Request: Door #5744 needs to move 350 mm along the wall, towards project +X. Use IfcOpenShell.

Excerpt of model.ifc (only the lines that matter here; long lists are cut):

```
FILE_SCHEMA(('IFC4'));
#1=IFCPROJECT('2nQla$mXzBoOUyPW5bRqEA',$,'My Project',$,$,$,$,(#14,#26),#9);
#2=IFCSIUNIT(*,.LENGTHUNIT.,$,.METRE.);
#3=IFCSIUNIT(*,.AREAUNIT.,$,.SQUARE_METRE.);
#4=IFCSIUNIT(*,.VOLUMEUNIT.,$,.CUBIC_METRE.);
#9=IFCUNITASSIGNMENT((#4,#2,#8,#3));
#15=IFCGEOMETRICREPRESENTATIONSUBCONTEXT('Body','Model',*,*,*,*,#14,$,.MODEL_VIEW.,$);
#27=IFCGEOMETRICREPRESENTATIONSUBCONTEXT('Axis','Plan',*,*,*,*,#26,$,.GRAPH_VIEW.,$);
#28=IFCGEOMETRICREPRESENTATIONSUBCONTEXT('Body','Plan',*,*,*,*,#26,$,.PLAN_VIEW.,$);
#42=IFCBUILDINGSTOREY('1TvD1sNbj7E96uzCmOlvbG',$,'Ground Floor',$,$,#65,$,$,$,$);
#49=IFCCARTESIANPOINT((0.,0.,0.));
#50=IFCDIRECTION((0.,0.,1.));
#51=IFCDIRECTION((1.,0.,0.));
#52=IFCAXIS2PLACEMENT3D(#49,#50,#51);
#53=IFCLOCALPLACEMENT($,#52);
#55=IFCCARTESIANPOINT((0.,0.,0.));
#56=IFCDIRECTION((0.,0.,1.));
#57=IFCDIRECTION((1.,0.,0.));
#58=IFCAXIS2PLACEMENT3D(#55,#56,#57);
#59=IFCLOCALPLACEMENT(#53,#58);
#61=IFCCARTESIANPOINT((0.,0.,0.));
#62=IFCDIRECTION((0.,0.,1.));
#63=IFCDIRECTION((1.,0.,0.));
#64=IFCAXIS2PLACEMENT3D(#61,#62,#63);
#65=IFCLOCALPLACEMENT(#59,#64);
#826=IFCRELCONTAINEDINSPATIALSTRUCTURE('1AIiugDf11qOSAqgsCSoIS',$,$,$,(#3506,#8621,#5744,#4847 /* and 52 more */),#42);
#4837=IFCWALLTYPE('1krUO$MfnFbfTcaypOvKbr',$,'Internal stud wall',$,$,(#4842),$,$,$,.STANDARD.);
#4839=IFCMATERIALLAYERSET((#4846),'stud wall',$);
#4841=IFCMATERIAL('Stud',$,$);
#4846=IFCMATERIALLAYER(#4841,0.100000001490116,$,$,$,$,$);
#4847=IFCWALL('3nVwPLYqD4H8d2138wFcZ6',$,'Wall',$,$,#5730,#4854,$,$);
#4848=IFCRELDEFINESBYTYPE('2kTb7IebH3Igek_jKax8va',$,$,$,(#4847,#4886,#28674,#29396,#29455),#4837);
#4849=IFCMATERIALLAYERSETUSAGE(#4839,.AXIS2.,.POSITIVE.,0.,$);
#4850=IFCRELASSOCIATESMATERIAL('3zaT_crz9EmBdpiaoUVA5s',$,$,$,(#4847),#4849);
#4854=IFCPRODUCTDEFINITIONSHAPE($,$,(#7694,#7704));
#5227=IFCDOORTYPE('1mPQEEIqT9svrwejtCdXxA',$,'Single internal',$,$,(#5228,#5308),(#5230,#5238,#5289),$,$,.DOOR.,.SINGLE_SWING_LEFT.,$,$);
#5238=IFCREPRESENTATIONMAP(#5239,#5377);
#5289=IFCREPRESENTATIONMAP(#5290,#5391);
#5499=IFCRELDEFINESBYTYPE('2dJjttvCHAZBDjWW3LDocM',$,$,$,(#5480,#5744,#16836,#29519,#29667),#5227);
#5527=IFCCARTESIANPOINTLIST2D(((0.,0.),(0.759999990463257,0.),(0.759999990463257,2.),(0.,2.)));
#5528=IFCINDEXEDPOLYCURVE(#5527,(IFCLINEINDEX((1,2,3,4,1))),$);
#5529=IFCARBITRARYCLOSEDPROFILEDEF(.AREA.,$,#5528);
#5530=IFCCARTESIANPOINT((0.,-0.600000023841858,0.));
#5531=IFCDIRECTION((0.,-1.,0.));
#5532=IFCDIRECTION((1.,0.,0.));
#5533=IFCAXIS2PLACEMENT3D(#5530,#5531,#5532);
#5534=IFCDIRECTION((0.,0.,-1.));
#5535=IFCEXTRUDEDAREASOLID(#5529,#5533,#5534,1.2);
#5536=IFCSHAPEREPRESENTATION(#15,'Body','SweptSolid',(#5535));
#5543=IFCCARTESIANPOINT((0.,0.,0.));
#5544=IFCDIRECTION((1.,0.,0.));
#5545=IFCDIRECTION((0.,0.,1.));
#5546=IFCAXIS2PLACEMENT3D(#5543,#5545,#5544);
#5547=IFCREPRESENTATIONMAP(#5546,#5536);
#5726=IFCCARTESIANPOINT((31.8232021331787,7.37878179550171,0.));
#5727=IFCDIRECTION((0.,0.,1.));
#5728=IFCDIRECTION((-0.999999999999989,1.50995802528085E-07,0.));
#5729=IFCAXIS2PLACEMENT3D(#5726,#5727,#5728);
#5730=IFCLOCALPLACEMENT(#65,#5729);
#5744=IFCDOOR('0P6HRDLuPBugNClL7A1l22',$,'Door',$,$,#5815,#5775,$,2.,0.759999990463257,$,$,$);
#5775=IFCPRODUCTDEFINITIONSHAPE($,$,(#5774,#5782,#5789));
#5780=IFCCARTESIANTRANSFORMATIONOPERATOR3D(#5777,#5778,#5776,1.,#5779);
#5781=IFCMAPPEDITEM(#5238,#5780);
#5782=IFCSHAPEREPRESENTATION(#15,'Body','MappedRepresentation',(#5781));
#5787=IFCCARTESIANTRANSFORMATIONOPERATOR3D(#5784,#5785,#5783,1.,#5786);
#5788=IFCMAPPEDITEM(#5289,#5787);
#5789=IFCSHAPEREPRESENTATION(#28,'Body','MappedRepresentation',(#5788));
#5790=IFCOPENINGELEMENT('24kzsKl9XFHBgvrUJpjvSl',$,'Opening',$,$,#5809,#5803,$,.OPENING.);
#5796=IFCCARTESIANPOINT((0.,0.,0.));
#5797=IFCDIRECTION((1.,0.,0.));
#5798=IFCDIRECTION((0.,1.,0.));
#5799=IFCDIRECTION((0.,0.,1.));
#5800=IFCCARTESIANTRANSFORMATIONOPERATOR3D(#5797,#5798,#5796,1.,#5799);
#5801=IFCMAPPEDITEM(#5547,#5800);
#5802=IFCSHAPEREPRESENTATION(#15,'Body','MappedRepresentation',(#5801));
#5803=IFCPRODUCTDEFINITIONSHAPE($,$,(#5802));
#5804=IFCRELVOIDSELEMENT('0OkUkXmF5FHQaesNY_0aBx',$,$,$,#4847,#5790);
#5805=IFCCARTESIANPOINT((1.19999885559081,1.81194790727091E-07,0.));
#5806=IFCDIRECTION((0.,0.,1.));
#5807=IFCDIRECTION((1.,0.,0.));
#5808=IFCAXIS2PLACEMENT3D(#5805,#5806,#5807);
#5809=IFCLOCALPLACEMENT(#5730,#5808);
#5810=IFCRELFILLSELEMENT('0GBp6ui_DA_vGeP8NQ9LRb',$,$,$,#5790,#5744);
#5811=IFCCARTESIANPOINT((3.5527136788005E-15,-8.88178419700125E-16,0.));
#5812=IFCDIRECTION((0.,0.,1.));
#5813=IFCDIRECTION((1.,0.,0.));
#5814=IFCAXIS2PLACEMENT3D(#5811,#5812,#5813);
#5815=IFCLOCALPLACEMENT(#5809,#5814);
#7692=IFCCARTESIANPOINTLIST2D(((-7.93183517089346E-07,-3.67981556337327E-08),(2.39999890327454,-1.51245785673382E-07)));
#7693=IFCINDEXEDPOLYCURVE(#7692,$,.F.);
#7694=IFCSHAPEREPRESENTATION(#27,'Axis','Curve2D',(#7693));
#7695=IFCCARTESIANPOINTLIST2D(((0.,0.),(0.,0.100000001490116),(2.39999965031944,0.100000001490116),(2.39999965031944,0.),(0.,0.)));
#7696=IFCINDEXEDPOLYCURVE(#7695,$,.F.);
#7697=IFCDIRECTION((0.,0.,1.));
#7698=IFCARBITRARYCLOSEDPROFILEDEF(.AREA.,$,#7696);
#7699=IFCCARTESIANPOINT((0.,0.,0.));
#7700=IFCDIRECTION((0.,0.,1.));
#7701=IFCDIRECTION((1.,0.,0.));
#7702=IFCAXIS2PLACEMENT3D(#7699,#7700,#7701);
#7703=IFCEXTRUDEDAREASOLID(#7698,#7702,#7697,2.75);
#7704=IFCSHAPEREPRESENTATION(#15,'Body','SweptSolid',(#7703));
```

```python
import ifcopenshell
import ifcopenshell.api.geometry
import ifcopenshell.util.placement

model = ifcopenshell.open("model.ifc")

door = model.by_guid("0P6HRDLuPBugNClL7A1l22")
opening = door.FillsVoids[0].RelatingOpeningElement
wall = opening.VoidsElements[0].RelatingBuildingElement

wall_matrix = ifcopenshell.util.placement.get_local_placement(wall.ObjectPlacement)
shift = wall_matrix[:3, 0] * -0.35
before = ifcopenshell.util.placement.get_local_placement(door.ObjectPlacement)[:3, 3].copy()

# The door is placed relative to its opening, so it follows when the opening moves.
matrix = ifcopenshell.util.placement.get_local_placement(opening.ObjectPlacement)
matrix[:3, 3] += shift
ifcopenshell.api.geometry.edit_object_placement(
    model, product=opening, matrix=matrix, is_si=False, should_transform_children=True
)

after = ifcopenshell.util.placement.get_local_placement(door.ObjectPlacement)[:3, 3]
print("door moved by", (after - before).round(3) + 0.0)

model.write("model_edited.ifc")
```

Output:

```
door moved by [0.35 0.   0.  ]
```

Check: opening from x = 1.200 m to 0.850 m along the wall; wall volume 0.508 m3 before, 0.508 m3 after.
